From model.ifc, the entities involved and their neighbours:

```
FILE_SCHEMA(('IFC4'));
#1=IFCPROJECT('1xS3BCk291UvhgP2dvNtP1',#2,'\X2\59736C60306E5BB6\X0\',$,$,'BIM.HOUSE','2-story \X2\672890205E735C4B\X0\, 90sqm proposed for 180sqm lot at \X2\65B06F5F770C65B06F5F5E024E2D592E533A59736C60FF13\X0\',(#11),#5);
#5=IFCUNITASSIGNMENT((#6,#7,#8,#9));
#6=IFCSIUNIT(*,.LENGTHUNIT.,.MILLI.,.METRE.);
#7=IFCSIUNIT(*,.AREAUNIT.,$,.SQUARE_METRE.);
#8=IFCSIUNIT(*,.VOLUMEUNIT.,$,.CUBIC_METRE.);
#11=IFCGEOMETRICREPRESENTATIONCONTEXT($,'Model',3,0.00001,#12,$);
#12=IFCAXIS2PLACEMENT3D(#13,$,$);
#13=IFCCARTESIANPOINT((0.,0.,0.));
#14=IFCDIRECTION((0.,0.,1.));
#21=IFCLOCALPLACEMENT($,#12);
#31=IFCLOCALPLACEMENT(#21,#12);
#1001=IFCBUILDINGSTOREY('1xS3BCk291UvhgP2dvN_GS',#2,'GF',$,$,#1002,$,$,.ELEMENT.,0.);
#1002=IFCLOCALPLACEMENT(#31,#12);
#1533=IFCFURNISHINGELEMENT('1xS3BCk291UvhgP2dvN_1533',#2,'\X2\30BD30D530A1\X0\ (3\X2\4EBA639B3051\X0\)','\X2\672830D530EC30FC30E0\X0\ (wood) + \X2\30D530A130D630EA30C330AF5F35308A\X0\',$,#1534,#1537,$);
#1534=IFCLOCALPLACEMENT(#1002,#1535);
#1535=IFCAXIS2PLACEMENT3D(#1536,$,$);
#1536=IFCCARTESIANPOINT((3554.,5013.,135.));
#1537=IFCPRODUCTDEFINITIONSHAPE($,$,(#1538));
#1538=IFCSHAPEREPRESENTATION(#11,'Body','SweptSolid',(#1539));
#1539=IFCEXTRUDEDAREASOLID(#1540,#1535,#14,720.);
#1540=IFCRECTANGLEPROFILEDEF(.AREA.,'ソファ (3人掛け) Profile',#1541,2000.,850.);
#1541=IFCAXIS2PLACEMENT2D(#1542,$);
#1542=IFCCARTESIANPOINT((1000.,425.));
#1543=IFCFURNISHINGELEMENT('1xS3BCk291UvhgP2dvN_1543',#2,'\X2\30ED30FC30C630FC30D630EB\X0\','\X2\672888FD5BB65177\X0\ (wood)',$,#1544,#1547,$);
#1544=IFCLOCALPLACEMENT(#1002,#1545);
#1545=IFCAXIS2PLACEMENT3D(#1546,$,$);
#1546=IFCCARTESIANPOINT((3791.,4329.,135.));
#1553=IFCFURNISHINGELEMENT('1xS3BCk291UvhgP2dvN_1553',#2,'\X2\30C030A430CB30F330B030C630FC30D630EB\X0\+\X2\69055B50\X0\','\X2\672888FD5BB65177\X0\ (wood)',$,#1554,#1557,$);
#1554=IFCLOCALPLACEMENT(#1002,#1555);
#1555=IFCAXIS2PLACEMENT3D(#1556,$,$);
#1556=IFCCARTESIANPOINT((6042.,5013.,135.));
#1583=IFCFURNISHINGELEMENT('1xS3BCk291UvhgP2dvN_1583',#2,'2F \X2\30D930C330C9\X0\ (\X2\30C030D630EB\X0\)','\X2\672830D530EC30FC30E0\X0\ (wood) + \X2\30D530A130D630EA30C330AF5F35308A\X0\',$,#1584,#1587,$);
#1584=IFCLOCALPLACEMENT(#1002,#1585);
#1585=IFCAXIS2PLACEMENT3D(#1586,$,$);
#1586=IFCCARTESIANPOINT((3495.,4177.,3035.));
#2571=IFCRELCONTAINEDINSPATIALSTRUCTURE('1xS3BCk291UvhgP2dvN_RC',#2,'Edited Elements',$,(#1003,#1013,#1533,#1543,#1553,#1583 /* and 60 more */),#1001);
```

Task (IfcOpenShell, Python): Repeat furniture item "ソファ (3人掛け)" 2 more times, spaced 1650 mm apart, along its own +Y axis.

```python
import ifcopenshell
import ifcopenshell.api.geometry
import ifcopenshell.api.root
import ifcopenshell.util.element
import ifcopenshell.util.placement

model = ifcopenshell.open("model.ifc")


def reuse_history(source, copy):
    """copy_class also copies each property set's owner history, people and application; keep the originals."""
    for rel in copy.IsDefinedBy:
        if rel.is_a("IfcRelDefinesByProperties") and (history := rel.RelatingPropertyDefinition.OwnerHistory):
            rel.RelatingPropertyDefinition.OwnerHistory = source.OwnerHistory
            ifcopenshell.util.element.remove_deep2(model, history)


source = model.by_guid("1xS3BCk291UvhgP2dvN_1533")
base = ifcopenshell.util.placement.get_local_placement(source.ObjectPlacement)
step = base[:3, 1] * 1650.0

for i in range(1, 3):
    copy = ifcopenshell.api.root.copy_class(model, product=source)
    copy.Representation = ifcopenshell.util.element.copy_deep(
        model, source.Representation, exclude=["IfcGeometricRepresentationContext", "IfcRepresentationMap"]
    )
    reuse_history(source, copy)
    matrix = base.copy()
    matrix[:3, 3] += i * step
    print("added at", matrix[:3, 3].round(3) + 0.0)
    ifcopenshell.api.geometry.edit_object_placement(model, product=copy, matrix=matrix, is_si=False)

model.write("model-out.ifc")
```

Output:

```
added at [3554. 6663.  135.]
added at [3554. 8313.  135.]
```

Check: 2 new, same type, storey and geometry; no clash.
